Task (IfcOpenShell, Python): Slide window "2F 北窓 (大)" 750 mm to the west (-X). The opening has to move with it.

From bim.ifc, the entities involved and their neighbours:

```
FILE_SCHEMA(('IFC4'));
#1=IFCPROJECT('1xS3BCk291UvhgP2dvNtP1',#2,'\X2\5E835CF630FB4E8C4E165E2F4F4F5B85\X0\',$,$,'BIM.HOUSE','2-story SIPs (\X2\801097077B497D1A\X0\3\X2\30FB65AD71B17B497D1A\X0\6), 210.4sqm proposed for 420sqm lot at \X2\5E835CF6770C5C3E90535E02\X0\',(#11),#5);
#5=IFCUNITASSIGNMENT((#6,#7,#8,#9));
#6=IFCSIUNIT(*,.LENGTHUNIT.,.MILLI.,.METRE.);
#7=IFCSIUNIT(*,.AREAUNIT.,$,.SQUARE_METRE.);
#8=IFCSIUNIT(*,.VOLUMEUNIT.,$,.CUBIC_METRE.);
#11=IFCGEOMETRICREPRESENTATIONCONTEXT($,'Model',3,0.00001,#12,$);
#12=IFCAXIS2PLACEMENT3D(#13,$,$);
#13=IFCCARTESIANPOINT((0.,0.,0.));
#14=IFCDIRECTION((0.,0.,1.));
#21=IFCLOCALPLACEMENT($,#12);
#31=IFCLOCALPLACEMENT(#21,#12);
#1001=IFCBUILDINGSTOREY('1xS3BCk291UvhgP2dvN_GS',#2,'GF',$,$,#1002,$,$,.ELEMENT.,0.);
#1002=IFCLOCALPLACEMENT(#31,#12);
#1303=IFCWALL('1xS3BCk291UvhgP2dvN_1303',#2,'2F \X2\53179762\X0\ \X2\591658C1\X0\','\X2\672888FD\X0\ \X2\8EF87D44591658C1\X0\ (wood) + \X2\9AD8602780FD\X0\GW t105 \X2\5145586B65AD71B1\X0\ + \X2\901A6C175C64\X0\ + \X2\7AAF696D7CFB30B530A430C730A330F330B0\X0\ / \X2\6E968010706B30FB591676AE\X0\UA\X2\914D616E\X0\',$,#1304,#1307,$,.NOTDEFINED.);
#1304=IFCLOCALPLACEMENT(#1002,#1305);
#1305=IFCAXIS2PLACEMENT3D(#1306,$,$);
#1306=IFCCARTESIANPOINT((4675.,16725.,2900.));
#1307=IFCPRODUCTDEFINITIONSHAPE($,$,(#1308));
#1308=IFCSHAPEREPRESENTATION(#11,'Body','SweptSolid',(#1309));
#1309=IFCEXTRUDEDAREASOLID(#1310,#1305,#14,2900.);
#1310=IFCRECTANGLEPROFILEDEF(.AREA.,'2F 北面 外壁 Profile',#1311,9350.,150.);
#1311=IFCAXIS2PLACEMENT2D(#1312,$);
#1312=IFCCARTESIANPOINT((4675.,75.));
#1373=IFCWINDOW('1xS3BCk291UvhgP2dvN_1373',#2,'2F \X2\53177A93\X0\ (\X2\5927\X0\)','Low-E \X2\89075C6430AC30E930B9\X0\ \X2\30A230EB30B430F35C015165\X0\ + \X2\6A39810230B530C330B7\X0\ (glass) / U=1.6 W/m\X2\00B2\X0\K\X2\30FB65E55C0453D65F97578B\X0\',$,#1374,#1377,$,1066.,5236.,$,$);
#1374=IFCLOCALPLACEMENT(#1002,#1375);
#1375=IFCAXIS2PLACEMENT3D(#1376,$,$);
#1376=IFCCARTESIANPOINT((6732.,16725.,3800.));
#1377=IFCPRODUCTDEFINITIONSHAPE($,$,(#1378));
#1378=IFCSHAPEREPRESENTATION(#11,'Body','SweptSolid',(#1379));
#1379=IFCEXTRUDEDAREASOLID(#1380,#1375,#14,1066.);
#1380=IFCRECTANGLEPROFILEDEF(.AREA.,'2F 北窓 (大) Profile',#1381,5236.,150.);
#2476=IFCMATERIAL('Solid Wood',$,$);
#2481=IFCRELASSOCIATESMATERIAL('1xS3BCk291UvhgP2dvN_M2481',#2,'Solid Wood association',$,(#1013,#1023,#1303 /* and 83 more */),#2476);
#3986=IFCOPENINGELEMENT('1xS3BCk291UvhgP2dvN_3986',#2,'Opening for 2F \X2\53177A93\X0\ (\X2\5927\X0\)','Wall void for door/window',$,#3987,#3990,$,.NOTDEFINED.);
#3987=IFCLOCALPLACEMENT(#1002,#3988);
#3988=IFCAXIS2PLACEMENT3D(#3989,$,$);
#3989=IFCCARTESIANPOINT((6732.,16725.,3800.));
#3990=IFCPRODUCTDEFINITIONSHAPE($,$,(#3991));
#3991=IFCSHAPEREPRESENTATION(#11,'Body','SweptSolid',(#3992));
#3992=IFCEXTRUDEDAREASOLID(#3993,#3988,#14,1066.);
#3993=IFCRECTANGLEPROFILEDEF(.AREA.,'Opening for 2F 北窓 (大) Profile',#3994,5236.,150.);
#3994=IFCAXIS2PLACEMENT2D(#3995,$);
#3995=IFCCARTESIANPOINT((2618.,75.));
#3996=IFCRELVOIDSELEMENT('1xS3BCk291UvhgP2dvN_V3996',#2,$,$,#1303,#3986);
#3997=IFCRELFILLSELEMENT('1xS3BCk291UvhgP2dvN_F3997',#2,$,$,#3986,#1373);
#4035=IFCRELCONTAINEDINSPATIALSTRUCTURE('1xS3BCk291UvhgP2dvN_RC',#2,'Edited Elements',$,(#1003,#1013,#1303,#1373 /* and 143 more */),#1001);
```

```python
import ifcopenshell
import ifcopenshell.api.geometry
import ifcopenshell.util.placement

model = ifcopenshell.open("bim.ifc")

window = model.by_guid("1xS3BCk291UvhgP2dvN_1373")
opening = window.FillsVoids[0].RelatingOpeningElement
wall = opening.VoidsElements[0].RelatingBuildingElement

wall_matrix = ifcopenshell.util.placement.get_local_placement(wall.ObjectPlacement)
shift = wall_matrix[:3, 0] * -750.0
before = ifcopenshell.util.placement.get_local_placement(window.ObjectPlacement)[:3, 3].copy()

# The window is not placed relative to its opening, so move both.
for product in (opening, window):
    matrix = ifcopenshell.util.placement.get_local_placement(product.ObjectPlacement)
    matrix[:3, 3] += shift
    ifcopenshell.api.geometry.edit_object_placement(model, product=product, matrix=matrix, is_si=False)

after = ifcopenshell.util.placement.get_local_placement(window.ObjectPlacement)[:3, 3]
print("window moved by", (after - before).round(3) + 0.0)

model.write("bim-out.ifc")
```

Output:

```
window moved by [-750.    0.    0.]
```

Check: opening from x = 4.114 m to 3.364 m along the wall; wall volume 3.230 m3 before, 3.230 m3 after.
